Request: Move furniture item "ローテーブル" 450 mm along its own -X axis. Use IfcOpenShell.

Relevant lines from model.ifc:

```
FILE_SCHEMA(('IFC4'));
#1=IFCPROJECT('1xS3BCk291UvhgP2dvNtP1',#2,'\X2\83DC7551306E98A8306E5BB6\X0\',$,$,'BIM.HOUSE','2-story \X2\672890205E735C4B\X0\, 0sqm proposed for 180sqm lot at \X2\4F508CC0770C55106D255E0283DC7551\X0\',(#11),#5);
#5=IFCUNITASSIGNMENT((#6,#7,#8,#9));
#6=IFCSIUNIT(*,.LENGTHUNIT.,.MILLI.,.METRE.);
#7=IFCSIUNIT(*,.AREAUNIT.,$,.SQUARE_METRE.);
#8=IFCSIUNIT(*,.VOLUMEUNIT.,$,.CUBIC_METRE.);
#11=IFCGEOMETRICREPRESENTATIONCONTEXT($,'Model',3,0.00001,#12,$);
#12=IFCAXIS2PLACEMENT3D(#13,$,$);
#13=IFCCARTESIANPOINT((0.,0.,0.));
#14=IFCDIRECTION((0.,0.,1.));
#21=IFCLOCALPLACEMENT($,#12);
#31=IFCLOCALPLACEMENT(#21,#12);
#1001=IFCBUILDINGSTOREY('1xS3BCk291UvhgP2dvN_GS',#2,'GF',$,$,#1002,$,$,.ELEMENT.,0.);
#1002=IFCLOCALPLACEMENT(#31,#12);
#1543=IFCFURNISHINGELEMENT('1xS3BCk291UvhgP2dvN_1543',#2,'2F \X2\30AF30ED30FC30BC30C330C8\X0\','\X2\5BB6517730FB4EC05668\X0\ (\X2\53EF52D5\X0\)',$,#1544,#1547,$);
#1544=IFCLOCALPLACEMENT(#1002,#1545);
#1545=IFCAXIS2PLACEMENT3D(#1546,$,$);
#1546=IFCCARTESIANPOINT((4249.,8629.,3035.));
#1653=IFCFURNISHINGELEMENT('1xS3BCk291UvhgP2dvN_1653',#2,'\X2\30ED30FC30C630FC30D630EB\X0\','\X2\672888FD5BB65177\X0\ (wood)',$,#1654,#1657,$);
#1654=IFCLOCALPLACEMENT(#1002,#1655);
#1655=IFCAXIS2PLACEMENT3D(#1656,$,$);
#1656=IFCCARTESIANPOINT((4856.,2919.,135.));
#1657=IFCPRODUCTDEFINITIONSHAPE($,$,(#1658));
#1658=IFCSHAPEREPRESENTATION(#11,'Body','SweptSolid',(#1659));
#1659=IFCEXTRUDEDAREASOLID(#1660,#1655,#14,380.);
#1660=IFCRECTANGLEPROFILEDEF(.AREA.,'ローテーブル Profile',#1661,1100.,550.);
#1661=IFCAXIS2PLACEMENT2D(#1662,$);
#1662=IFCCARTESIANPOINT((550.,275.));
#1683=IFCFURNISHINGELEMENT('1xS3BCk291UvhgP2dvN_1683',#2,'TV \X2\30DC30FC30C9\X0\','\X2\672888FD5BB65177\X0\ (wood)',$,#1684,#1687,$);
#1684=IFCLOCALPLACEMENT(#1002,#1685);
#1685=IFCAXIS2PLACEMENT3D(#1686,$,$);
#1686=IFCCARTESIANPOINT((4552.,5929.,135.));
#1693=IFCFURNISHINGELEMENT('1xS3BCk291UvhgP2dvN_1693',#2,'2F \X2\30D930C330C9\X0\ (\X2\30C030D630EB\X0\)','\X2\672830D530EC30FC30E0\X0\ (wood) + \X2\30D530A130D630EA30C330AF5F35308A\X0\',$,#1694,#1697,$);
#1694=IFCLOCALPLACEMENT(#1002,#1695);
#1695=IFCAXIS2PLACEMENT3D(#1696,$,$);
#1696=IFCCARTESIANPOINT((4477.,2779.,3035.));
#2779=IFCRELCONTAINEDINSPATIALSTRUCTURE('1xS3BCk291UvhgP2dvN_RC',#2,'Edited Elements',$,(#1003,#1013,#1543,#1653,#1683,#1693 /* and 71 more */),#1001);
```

```python
import ifcopenshell
import ifcopenshell.api.geometry
import ifcopenshell.util.placement
import ifcopenshell.util.unit

model = ifcopenshell.open("model.ifc")
unit_scale = ifcopenshell.util.unit.calculate_unit_scale(model)

item = model.by_guid("1xS3BCk291UvhgP2dvN_1653")
matrix = ifcopenshell.util.placement.get_local_placement(item.ObjectPlacement)
matrix[:3, 3] -= matrix[:3, 0] * 0.45 / unit_scale
ifcopenshell.api.geometry.edit_object_placement(model, product=item, matrix=matrix, is_si=False)

print(ifcopenshell.util.placement.get_local_placement(item.ObjectPlacement).round(3) + 0.0)

model.write("model-out.ifc")
```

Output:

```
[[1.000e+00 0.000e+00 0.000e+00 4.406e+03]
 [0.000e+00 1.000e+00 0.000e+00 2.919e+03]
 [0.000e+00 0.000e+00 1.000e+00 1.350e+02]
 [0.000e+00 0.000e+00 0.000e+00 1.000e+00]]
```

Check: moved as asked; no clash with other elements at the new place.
